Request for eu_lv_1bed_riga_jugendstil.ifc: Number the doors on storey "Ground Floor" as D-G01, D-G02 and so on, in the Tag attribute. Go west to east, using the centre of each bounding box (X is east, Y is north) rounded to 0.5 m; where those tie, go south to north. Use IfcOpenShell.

First a look at what the model holds.

```python
import ifcopenshell
import ifcopenshell.util.element
import ifcopenshell.util.placement

model = ifcopenshell.open("eu_lv_1bed_riga_jugendstil.ifc")
print(model.schema)
storey = next(s for s in model.by_type("IfcBuildingStorey") if s.Name == "Ground Floor")
doors = [e for e in ifcopenshell.util.element.get_decomposition(storey) if e.is_a("IfcDoor")]
for e in sorted(doors, key=lambda e: e.id()):
    origin = ifcopenshell.util.placement.get_local_placement(e.ObjectPlacement)[:3, 3]
    print(e.id(), e.Tag, e.Name, origin.round(2) + 0.0, sep=" | ")
```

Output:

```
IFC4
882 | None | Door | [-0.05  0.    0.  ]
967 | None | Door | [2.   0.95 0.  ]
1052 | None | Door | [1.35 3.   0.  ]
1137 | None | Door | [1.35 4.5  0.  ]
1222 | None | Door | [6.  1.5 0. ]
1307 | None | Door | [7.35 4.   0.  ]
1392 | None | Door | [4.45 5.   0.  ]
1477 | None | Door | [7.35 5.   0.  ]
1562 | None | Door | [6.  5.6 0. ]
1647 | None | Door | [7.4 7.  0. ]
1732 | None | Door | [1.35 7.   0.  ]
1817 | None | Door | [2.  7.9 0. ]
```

```python
import ifcopenshell
import ifcopenshell.geom
import ifcopenshell.util.element
import ifcopenshell.util.shape

model = ifcopenshell.open("eu_lv_1bed_riga_jugendstil.ifc")
settings = ifcopenshell.geom.settings()
settings.set("use-world-coords", True)


def centre(element):
    shape = ifcopenshell.geom.create_shape(settings, element)
    return ifcopenshell.util.shape.get_bbox_centroid(shape.geometry)


storey = next(s for s in model.by_type("IfcBuildingStorey") if s.Name == "Ground Floor")
doors = [e for e in ifcopenshell.util.element.get_decomposition(storey) if e.is_a("IfcDoor")]

# Insertion points can sit at a corner or the storey origin, so sort by the geometry (in metres).
centres = {e: centre(e) for e in doors}
doors.sort(key=lambda e: (round(centres[e][0] / 0.5), centres[e][1]))

for i, e in enumerate(doors, start=1):
    number = f"D-G{i:02d}"
    e.Tag = number
    print(e.id(), number)

model.write("eu_lv_1bed_riga_jugendstil_updated.ifc")
```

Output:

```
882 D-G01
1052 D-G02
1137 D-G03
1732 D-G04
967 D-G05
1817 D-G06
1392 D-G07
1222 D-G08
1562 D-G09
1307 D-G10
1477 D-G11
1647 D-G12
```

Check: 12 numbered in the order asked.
